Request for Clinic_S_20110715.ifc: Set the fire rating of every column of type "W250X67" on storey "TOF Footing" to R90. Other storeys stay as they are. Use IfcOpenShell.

First a look at what the model holds.

```python
import ifcopenshell
import ifcopenshell.util.element

model = ifcopenshell.open("Clinic_S_20110715.ifc")
print(model.schema)
storey = next(s for s in model.by_type("IfcBuildingStorey") if s.Name == "TOF Footing")
columns = [e for e in ifcopenshell.util.element.get_decomposition(storey) if e.is_a("IfcColumn")]
seen = {}
for e in columns:
    element_type = ifcopenshell.util.element.get_type(e)
    key = (element_type.Name if element_type != e and element_type else None, ifcopenshell.util.element.get_pset(e, "Pset_ColumnCommon", "FireRating"))
    seen[key] = seen.get(key, 0) + 1
for (name, value), count in sorted(seen.items(), key=str):
    print(count, "x", name, "|", value)
```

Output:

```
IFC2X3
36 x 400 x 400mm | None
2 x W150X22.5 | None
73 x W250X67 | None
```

```python
import ifcopenshell
import ifcopenshell.api.pset
import ifcopenshell.util.element

model = ifcopenshell.open("Clinic_S_20110715.ifc")

storey = next(s for s in model.by_type("IfcBuildingStorey") if s.Name == "TOF Footing")
columns = [e for e in ifcopenshell.util.element.get_decomposition(storey) if e.is_a("IfcColumn")]

count = 0
for e in columns:
    element_type = ifcopenshell.util.element.get_type(e)
    if element_type in (None, e) or element_type.Name != "W250X67":
        continue
    # add_pset returns the element's existing set when there is one.
    pset = ifcopenshell.api.pset.add_pset(model, product=e, name="Pset_ColumnCommon")
    ifcopenshell.api.pset.edit_pset(model, pset=pset, properties={"FireRating": "R90"})
    count += 1

print(count, "columns updated")

model.write("Clinic_S_20110715_edited.ifc")
```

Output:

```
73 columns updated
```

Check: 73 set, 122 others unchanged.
